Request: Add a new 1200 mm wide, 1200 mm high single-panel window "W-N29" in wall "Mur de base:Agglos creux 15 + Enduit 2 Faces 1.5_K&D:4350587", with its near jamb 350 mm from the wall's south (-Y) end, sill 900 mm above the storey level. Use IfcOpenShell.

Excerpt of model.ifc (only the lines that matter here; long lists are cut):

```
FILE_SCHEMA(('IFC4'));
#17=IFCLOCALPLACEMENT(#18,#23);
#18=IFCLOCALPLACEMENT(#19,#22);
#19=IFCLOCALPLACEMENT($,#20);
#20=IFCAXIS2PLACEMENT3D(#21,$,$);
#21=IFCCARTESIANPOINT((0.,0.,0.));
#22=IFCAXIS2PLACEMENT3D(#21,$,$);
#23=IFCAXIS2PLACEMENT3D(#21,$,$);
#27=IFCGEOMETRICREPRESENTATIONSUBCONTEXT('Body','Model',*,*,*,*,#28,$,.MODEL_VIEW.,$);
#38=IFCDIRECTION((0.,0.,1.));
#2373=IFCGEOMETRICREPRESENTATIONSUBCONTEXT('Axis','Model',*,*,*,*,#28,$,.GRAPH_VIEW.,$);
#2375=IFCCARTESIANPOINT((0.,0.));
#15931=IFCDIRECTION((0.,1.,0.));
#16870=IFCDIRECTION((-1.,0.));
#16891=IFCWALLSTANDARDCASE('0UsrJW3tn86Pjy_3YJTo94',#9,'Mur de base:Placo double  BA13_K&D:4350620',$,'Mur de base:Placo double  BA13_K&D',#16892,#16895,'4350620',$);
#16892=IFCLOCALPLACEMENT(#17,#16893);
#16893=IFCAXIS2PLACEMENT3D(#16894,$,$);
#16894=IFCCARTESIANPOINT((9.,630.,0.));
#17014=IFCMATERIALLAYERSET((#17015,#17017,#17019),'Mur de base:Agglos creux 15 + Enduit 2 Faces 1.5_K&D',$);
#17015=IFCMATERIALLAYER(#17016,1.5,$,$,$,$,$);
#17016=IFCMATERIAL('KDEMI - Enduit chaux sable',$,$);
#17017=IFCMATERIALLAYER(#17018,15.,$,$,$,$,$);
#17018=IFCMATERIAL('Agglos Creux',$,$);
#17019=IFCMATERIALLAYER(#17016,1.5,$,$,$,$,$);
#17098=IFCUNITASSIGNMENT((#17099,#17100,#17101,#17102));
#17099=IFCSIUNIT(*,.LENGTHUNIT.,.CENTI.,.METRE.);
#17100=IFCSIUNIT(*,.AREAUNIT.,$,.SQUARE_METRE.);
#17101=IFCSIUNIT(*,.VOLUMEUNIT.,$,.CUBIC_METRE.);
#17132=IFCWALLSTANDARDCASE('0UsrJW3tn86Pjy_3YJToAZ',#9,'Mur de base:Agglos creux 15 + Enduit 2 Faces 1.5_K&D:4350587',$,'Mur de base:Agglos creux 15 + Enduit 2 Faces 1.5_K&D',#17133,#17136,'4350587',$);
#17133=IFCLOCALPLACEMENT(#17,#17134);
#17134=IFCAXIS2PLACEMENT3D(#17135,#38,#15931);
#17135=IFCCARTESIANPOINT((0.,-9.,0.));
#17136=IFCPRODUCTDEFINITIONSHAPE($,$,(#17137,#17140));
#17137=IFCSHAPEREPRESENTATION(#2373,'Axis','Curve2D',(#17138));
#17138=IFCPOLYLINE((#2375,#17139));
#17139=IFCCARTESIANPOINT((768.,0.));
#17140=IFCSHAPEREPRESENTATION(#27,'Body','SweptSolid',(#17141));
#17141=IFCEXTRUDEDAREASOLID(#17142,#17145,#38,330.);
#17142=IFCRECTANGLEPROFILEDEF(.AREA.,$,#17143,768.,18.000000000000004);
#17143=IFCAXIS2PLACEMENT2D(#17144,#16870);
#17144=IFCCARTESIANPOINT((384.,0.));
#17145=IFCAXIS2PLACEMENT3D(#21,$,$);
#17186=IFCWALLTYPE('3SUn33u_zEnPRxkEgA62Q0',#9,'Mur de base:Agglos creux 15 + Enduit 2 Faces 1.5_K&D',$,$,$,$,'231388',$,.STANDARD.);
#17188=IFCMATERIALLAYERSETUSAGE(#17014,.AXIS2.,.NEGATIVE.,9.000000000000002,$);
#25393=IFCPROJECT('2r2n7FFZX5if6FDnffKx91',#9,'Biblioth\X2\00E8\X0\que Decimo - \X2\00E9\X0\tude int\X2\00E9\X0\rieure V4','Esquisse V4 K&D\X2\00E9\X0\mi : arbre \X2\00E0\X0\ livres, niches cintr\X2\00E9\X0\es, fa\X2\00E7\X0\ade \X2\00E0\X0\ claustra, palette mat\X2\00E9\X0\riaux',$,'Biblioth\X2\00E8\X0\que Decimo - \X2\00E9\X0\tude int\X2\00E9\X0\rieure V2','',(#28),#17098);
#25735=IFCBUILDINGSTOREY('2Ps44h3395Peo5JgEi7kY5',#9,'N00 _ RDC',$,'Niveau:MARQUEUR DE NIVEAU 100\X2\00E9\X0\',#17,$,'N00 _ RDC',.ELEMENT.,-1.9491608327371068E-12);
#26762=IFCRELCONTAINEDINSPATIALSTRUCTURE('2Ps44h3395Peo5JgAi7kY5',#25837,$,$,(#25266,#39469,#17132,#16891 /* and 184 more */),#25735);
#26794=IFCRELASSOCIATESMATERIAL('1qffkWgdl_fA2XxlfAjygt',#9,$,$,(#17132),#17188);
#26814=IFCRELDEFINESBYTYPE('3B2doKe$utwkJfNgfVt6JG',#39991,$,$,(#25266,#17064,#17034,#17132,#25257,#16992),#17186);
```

```python
import numpy as np
import ifcopenshell
import ifcopenshell.api.feature
import ifcopenshell.api.geometry
import ifcopenshell.api.root
import ifcopenshell.api.spatial
import ifcopenshell.geom
import ifcopenshell.util.element
import ifcopenshell.util.placement
import ifcopenshell.util.representation
import ifcopenshell.util.shape
import ifcopenshell.util.unit

model = ifcopenshell.open("model.ifc")
unit_scale = ifcopenshell.util.unit.calculate_unit_scale(model)
settings = ifcopenshell.geom.settings()


def volume(element):
    """Net volume in cubic metres, openings subtracted."""
    shape = ifcopenshell.geom.create_shape(settings, element)
    return ifcopenshell.util.shape.get_volume(shape.geometry)


wall = model.by_guid("0UsrJW3tn86Pjy_3YJToAZ")
storey = ifcopenshell.util.element.get_container(wall, ifc_class="IfcBuildingStorey")
context = ifcopenshell.util.representation.get_context(model, "Model", "Body", "MODEL_VIEW")
before = volume(wall)

width, height, from_end, sill = 1.2, 1.2, 0.35, 0.9  # metres

# The wall runs along its own X axis, and the end named is its -X end.
wall_shape = ifcopenshell.geom.create_shape(settings, wall)
x, y, z = ifcopenshell.util.shape.get_vertices(wall_shape.geometry).T
start = x.min() + from_end
face, thickness = float(y.min()), float(y.max() - y.min())
wall_matrix = ifcopenshell.util.placement.get_local_placement(wall.ObjectPlacement)
level = ifcopenshell.util.placement.get_local_placement(storey.ObjectPlacement)[2, 3]


def in_wall(x, y):
    """Placement at x, y metres in the wall's axes, at sill height."""
    matrix = wall_matrix.copy()
    matrix[:, 3] = wall_matrix @ np.array([x / unit_scale, y / unit_scale, 0.0, 1.0])
    matrix[2, 3] = level + sill / unit_scale
    return matrix


# Opening: a box that overshoots both wall faces by 50 mm.
opening = ifcopenshell.api.root.create_entity(model, ifc_class="IfcOpeningElement", predefined_type="OPENING")
box = ifcopenshell.api.geometry.add_wall_representation(
    model, context=context, length=width, height=height, thickness=thickness + 0.1
)
ifcopenshell.api.geometry.assign_representation(model, product=opening, representation=box)
ifcopenshell.api.geometry.edit_object_placement(model, product=opening, matrix=in_wall(start, face - 0.05), is_si=False)
ifcopenshell.api.feature.add_feature(model, feature=opening, element=wall)

window = ifcopenshell.api.root.create_entity(model, ifc_class="IfcWindow", name="W-N29", predefined_type="WINDOW")
window.OverallWidth, window.OverallHeight = width / unit_scale, height / unit_scale
window.PartitioningType = "SINGLE_PANEL"
body = ifcopenshell.api.geometry.add_window_representation(
    model,
    context=context,
    overall_width=window.OverallWidth,
    overall_height=window.OverallHeight,
    partition_type="SINGLE_PANEL",
)
ifcopenshell.api.geometry.assign_representation(model, product=window, representation=body)
ifcopenshell.api.spatial.assign_container(model, products=[window], relating_structure=storey)
ifcopenshell.api.feature.add_filling(model, opening=opening, element=window)

# Centre the window in the wall's thickness.
ifcopenshell.api.geometry.edit_object_placement(model, product=window, matrix=in_wall(start, face), is_si=False)
window_shape = ifcopenshell.geom.create_shape(settings, window)
depth = ifcopenshell.util.shape.get_vertices(window_shape.geometry)[:, 1]
offset = face + thickness / 2 - (depth.min() + depth.max()) / 2
ifcopenshell.api.geometry.edit_object_placement(model, product=window, matrix=in_wall(start, offset), is_si=False)

after = volume(wall)

print(f"wall volume {before:.3f} -> {after:.3f} m3")

model.write("model_rev.ifc")
```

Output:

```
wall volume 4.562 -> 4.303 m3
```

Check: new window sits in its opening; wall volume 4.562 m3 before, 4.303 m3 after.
